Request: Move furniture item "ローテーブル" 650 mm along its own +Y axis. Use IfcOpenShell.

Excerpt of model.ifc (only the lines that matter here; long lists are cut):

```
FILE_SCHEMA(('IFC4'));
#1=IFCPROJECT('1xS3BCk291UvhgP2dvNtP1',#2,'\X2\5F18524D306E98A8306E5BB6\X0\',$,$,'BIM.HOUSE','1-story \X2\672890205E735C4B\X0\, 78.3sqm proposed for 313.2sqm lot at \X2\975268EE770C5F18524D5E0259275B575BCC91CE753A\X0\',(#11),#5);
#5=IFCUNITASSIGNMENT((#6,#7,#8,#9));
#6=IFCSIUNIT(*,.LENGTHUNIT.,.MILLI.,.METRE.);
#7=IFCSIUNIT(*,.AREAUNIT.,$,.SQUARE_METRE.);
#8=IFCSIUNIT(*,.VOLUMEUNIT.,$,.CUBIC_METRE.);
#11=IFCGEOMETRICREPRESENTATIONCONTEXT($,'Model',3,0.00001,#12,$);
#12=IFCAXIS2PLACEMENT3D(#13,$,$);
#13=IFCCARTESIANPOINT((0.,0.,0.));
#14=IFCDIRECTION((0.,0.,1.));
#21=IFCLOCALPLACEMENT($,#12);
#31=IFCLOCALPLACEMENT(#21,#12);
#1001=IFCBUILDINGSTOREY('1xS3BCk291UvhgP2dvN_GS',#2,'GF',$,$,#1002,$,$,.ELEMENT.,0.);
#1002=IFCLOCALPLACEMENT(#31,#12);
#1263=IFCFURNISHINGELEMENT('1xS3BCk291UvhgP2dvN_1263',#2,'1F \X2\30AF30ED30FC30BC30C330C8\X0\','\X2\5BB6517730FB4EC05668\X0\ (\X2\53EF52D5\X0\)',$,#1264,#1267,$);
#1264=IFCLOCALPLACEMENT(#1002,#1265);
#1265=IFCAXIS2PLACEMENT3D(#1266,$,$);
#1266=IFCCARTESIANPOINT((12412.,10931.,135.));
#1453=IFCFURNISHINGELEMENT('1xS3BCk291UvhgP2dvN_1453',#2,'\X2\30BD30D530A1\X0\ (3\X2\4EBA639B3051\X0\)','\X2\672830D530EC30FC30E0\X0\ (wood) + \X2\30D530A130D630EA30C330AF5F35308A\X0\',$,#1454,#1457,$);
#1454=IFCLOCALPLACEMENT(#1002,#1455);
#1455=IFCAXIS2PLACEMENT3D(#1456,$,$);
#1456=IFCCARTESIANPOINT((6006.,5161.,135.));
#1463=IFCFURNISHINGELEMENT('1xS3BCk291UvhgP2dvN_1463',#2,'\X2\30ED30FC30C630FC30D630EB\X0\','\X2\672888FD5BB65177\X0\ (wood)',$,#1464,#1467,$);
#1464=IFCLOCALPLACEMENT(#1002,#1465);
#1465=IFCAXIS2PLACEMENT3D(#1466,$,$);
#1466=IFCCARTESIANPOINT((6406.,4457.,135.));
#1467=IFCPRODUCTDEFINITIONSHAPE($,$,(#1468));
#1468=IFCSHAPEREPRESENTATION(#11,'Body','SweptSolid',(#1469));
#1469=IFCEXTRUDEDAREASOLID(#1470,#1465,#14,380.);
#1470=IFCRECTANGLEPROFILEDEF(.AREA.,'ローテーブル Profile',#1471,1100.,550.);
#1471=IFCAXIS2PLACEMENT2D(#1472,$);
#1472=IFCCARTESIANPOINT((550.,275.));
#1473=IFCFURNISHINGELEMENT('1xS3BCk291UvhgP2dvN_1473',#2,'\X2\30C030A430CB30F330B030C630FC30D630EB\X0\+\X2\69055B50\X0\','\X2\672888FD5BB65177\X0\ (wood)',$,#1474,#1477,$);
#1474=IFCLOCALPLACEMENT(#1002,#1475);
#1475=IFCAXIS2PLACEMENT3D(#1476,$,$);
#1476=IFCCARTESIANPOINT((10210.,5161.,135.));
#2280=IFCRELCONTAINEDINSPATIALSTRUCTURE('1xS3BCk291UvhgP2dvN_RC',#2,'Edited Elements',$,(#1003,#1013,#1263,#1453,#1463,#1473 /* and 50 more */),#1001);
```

```python
import ifcopenshell
import ifcopenshell.api.geometry
import ifcopenshell.util.placement

model = ifcopenshell.open("model.ifc")

item = model.by_guid("1xS3BCk291UvhgP2dvN_1463")
matrix = ifcopenshell.util.placement.get_local_placement(item.ObjectPlacement)
matrix[:3, 3] += matrix[:3, 1] * 650.0
ifcopenshell.api.geometry.edit_object_placement(model, product=item, matrix=matrix, is_si=False)

print(ifcopenshell.util.placement.get_local_placement(item.ObjectPlacement).round(3) + 0.0)

model.write("model_updated.ifc")
```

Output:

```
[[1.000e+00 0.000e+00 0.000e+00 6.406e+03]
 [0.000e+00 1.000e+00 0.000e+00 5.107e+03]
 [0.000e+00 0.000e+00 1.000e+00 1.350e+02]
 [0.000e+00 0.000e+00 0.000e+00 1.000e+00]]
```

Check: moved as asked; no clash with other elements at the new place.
